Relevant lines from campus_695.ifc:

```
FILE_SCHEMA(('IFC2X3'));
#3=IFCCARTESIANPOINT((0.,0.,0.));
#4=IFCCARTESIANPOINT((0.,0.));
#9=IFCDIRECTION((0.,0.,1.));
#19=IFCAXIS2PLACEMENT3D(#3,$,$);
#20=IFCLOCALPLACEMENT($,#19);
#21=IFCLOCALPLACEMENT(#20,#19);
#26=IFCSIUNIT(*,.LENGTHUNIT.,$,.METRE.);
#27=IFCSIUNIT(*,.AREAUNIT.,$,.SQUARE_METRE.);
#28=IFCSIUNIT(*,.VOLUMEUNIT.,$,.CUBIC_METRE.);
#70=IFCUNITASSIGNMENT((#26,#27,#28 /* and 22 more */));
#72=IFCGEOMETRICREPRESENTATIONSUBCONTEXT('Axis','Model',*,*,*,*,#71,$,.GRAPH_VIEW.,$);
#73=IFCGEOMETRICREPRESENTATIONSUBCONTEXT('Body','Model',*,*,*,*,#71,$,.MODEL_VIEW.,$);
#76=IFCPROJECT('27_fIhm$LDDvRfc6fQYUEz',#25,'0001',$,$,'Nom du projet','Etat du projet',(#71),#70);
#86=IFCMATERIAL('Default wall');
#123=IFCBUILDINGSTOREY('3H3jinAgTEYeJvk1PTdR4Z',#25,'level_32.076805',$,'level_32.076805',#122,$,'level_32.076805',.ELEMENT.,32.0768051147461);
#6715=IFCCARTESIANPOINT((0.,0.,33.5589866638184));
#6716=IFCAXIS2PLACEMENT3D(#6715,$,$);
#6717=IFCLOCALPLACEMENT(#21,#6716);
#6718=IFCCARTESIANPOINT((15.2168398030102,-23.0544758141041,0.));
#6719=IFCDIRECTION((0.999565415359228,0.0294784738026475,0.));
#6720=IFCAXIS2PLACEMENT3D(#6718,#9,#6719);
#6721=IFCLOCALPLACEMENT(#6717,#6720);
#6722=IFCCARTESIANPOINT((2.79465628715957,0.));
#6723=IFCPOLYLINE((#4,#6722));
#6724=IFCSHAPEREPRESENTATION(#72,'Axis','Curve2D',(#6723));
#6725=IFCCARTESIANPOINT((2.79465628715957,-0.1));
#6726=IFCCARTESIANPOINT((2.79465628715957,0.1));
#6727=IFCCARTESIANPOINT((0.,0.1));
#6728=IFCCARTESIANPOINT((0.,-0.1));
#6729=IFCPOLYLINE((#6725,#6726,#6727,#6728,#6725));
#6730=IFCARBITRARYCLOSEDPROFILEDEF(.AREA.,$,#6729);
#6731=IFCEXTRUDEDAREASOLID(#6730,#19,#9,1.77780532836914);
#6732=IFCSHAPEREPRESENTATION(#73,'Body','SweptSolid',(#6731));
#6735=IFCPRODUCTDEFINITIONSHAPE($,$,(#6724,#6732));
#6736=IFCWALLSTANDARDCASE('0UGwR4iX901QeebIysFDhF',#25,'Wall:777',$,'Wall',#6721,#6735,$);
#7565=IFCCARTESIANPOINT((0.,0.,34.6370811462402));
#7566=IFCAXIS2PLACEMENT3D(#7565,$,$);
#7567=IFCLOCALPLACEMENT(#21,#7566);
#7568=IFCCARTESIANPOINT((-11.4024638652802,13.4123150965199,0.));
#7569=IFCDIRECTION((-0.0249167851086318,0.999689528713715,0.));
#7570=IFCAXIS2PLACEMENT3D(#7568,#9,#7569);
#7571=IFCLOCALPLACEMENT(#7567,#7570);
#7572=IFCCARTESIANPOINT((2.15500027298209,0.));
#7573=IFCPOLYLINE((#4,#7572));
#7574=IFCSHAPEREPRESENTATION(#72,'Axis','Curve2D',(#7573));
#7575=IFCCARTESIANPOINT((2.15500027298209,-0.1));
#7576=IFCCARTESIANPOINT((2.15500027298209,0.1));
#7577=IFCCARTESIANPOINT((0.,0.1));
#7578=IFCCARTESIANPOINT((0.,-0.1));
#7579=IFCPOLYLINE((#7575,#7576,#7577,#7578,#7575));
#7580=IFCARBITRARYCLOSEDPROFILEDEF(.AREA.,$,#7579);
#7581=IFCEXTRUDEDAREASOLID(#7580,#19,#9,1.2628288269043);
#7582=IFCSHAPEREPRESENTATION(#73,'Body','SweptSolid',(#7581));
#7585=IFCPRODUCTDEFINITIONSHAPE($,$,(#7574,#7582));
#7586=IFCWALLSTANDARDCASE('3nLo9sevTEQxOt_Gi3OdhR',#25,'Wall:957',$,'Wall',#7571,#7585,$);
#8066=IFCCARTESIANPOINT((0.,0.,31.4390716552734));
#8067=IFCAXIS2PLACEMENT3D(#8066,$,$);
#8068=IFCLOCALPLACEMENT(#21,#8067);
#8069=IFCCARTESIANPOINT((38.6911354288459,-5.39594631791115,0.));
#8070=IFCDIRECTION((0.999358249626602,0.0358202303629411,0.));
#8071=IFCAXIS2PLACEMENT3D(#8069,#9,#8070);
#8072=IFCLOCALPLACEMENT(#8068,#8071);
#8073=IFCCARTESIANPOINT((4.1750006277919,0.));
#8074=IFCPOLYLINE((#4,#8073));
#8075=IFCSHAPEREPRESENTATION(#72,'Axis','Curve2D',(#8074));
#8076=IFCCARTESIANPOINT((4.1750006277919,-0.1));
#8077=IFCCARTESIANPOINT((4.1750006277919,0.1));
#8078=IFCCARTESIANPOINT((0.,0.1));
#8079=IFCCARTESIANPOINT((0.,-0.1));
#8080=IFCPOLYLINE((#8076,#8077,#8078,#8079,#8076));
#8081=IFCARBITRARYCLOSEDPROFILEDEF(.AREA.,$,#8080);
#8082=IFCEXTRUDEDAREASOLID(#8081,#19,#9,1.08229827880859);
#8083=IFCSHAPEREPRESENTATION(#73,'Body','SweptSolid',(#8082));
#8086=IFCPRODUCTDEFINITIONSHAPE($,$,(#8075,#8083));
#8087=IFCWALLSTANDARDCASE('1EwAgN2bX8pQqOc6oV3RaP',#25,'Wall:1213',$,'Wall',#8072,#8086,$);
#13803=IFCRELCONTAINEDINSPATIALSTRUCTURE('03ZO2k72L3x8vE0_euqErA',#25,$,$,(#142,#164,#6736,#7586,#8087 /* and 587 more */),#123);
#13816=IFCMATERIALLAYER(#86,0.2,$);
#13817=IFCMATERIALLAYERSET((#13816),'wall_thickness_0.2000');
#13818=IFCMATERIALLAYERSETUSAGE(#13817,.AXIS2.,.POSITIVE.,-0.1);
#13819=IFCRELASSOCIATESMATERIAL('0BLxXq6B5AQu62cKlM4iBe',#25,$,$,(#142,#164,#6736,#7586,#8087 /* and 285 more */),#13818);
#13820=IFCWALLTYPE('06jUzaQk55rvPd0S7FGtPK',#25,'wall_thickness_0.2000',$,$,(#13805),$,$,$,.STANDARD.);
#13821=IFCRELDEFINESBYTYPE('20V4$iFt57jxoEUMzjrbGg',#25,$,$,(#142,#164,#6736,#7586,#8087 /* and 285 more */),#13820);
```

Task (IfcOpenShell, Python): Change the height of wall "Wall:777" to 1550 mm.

```python
import ifcopenshell
import ifcopenshell.geom
import ifcopenshell.util.representation
import ifcopenshell.util.shape
import ifcopenshell.util.unit

model = ifcopenshell.open("campus_695.ifc")
unit_scale = ifcopenshell.util.unit.calculate_unit_scale(model)
settings = ifcopenshell.geom.settings()


def volume(element):
    """Net volume in cubic metres, openings subtracted."""
    shape = ifcopenshell.geom.create_shape(settings, element)
    return ifcopenshell.util.shape.get_volume(shape.geometry)


wall = model.by_guid("0UGwR4iX901QeebIysFDhF")
before = volume(wall)

body = ifcopenshell.util.representation.get_representation(wall, "Model", "Body")
solid = body.Items[0]
old_height = solid.Depth
solid.Depth = 1.55 / unit_scale
after = volume(wall)

print(f"height {old_height:g} -> {solid.Depth:g}, volume {before:.3f} -> {after:.3f} m3")

model.write("campus_695_rev.ifc")
```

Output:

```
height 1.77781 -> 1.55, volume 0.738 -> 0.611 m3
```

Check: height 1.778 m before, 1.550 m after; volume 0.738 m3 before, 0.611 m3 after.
